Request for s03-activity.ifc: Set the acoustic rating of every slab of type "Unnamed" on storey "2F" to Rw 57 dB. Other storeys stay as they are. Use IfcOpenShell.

First a look at what the model holds.

```python
import ifcopenshell
import ifcopenshell.util.element

model = ifcopenshell.open("s03-activity.ifc")
print(model.schema)
storey = next(s for s in model.by_type("IfcBuildingStorey") if s.Name == "2F")
slabs = [e for e in ifcopenshell.util.element.get_decomposition(storey) if e.is_a("IfcSlab")]
seen = {}
for e in slabs:
    element_type = ifcopenshell.util.element.get_type(e)
    key = (element_type.Name if element_type != e and element_type else None, ifcopenshell.util.element.get_pset(e, "Pset_SlabCommon", "AcousticRating"))
    seen[key] = seen.get(key, 0) + 1
for (name, value), count in sorted(seen.items(), key=str):
    print(count, "x", name, "|", value)
```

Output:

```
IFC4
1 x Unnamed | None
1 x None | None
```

```python
import ifcopenshell
import ifcopenshell.api.pset
import ifcopenshell.util.element

model = ifcopenshell.open("s03-activity.ifc")

storey = next(s for s in model.by_type("IfcBuildingStorey") if s.Name == "2F")
slabs = [e for e in ifcopenshell.util.element.get_decomposition(storey) if e.is_a("IfcSlab")]

count = 0
for e in slabs:
    element_type = ifcopenshell.util.element.get_type(e)
    if element_type in (None, e) or element_type.Name != "Unnamed":
        continue
    # add_pset returns the element's existing set when there is one.
    pset = ifcopenshell.api.pset.add_pset(model, product=e, name="Pset_SlabCommon")
    ifcopenshell.api.pset.edit_pset(model, pset=pset, properties={"AcousticRating": "Rw 57 dB"})
    count += 1

print(count, "slabs updated")

model.write("s03-activity_v2.ifc")
```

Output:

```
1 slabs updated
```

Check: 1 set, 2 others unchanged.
